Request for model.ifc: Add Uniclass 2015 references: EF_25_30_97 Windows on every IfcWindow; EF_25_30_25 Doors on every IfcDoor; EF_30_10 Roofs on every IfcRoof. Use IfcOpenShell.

First a look at what the model holds.

```python
import ifcopenshell

model = ifcopenshell.open("model.ifc")
print(model.schema)
print("classifications:", [c.Name for c in model.by_type("IfcClassification")])
for ifc_class in ("IfcDoor", "IfcRoof", "IfcStair", "IfcWall", "IfcWindow"):
    print(ifc_class, len(model.by_type(ifc_class)))
```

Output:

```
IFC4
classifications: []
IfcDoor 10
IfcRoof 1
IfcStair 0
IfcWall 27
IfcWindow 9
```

```python
import ifcopenshell
import ifcopenshell.api.classification

model = ifcopenshell.open("model.ifc")

system = ifcopenshell.api.classification.add_classification(model, classification="Uniclass 2015")

codes = {
    "IfcWindow": ("EF_25_30_97", "Windows"),
    "IfcDoor": ("EF_25_30_25", "Doors"),
    "IfcRoof": ("EF_30_10", "Roofs"),
}
for ifc_class, (code, name) in codes.items():
    products = model.by_type(ifc_class)
    ifcopenshell.api.classification.add_reference(
        model, products=products, classification=system, identification=code, name=name
    )
    print(code, len(products))

model.write("model_v2.ifc")
```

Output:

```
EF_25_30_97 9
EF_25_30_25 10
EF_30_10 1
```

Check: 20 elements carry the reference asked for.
